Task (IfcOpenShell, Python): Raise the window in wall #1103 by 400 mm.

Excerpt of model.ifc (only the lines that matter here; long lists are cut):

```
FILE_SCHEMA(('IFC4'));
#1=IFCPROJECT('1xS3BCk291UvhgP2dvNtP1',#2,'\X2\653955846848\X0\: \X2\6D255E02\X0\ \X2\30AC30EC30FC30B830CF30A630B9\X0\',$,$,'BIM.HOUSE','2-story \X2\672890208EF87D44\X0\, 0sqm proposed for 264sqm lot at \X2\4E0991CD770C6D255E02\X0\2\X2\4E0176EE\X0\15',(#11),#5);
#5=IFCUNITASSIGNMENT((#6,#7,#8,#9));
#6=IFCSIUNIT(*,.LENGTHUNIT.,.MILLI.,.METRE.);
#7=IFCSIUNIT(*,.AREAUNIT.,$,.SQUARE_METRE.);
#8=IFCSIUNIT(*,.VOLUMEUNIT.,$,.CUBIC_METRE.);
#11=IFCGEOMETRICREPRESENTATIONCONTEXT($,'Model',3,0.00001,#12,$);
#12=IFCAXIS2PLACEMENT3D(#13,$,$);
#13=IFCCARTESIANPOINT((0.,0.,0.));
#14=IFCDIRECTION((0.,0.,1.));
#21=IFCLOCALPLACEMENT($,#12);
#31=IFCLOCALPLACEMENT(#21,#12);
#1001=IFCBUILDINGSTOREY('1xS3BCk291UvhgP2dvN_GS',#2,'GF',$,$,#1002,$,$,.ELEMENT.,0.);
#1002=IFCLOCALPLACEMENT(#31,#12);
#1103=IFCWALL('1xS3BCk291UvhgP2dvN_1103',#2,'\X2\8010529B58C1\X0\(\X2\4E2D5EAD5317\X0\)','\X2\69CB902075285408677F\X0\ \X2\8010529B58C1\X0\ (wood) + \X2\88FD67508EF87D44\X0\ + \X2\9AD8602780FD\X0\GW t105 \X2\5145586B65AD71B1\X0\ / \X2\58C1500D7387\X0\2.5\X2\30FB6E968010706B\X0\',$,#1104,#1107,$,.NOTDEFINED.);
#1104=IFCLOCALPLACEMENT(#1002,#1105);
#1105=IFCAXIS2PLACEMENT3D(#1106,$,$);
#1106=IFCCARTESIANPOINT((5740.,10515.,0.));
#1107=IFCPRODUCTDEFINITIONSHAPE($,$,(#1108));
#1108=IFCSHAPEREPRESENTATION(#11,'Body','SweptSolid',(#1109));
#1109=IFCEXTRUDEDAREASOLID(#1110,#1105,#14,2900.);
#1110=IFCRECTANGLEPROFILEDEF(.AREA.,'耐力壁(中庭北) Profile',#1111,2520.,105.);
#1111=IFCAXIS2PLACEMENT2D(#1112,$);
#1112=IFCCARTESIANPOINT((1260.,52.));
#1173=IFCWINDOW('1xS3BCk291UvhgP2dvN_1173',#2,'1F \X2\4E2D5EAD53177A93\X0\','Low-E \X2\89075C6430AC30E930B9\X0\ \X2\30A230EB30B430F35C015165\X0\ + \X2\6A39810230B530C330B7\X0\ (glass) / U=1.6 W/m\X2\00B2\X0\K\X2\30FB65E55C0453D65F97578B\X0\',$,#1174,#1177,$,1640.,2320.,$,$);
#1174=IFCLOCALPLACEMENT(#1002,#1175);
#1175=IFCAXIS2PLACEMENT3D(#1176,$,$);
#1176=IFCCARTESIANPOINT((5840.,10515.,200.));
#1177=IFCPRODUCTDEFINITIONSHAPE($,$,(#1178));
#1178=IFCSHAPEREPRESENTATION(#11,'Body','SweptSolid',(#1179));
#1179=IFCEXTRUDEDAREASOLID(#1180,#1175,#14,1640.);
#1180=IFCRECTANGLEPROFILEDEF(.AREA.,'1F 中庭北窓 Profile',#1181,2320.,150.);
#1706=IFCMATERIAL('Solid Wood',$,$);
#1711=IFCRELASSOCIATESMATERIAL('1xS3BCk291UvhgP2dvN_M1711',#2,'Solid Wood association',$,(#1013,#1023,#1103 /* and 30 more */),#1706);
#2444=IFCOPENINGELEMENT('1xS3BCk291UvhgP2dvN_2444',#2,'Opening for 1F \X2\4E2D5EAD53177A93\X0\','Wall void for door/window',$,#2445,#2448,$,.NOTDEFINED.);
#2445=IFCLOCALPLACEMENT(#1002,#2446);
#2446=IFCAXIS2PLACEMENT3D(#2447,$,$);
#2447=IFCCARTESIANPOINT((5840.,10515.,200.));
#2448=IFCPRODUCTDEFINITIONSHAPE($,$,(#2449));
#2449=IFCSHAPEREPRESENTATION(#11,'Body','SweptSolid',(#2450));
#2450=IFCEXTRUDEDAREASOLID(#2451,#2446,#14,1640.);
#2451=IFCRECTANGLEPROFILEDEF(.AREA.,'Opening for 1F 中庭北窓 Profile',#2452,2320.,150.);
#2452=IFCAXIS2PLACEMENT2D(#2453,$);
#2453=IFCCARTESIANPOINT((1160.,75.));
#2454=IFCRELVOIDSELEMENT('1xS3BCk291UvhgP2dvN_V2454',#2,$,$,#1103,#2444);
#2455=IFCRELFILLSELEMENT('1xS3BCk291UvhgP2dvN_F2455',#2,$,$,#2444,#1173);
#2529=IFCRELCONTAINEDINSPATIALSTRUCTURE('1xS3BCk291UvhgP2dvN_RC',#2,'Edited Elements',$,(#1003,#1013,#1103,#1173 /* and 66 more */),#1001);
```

```python
import numpy as np
import ifcopenshell
import ifcopenshell.api.geometry
import ifcopenshell.util.placement
import ifcopenshell.util.unit

model = ifcopenshell.open("model.ifc")
unit_scale = ifcopenshell.util.unit.calculate_unit_scale(model)

window = model.by_guid("1xS3BCk291UvhgP2dvN_1173")
opening = window.FillsVoids[0].RelatingOpeningElement
dz = 0.4 / unit_scale

shift = np.array([0.0, 0.0, dz])
# The window is not placed relative to its opening, so move both.
for product in (opening, window):
    matrix = ifcopenshell.util.placement.get_local_placement(product.ObjectPlacement)
    matrix[:3, 3] += shift
    ifcopenshell.api.geometry.edit_object_placement(model, product=product, matrix=matrix, is_si=False)

print(f"moved by {dz * unit_scale:+.3f} m")

model.write("model_rev.ifc")
```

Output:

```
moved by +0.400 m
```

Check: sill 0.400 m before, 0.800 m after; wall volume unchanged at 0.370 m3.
